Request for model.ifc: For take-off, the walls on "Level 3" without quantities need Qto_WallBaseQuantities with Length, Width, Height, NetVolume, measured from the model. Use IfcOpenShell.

First a look at what the model holds.

```python
import ifcopenshell
import ifcopenshell.util.element
import ifcopenshell.util.unit

model = ifcopenshell.open("model.ifc")
print(model.schema)
for unit_type in ("LENGTHUNIT", "AREAUNIT", "VOLUMEUNIT"):
    print(unit_type, ifcopenshell.util.unit.calculate_unit_scale(model, unit_type))
storey = next(s for s in model.by_type("IfcBuildingStorey") if s.Name == "Level 3")
walls = [e for e in ifcopenshell.util.element.get_decomposition(storey) if e.is_a("IfcWall")]
for e in sorted(walls, key=lambda e: e.id()):
    print(e.id(), e.is_a(), e.Name, list(ifcopenshell.util.element.get_psets(e, qtos_only=True)), sep=" | ")
```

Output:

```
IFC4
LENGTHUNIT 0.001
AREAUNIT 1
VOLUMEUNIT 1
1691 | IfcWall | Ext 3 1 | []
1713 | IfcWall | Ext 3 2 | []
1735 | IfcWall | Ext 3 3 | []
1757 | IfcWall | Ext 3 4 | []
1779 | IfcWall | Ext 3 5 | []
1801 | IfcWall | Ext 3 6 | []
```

```python
import ifcopenshell
import ifcopenshell.api.pset
import ifcopenshell.geom
import ifcopenshell.util.element
import ifcopenshell.util.shape
import ifcopenshell.util.unit

model = ifcopenshell.open("model.ifc")
unit_scale = ifcopenshell.util.unit.calculate_unit_scale(model)
volume_scale = ifcopenshell.util.unit.calculate_unit_scale(model, "VOLUMEUNIT")
settings = ifcopenshell.geom.settings()

storey = next(s for s in model.by_type("IfcBuildingStorey") if s.Name == "Level 3")
walls = [e for e in ifcopenshell.util.element.get_decomposition(storey) if e.is_a("IfcWall")]

for e in sorted(walls, key=lambda e: e.id()):
    if ifcopenshell.util.element.get_psets(e, qtos_only=True, should_inherit=False):
        continue
    # Geometry comes back in metres, in the element's own axes.
    shape = ifcopenshell.geom.create_shape(settings, e)
    values = {
        "Length": ifcopenshell.util.shape.get_x(shape.geometry) / unit_scale,
        "Width": ifcopenshell.util.shape.get_y(shape.geometry) / unit_scale,
        "Height": ifcopenshell.util.shape.get_z(shape.geometry) / unit_scale,
        "NetVolume": ifcopenshell.util.shape.get_volume(shape.geometry) / volume_scale,
    }
    qto = ifcopenshell.api.pset.add_qto(model, product=e, name="Qto_WallBaseQuantities")
    ifcopenshell.api.pset.edit_qto(model, qto=qto, properties=values)
    print(e.id(), {k: round(v, 3) for k, v in values.items()})

model.write("model_rev.ifc")
```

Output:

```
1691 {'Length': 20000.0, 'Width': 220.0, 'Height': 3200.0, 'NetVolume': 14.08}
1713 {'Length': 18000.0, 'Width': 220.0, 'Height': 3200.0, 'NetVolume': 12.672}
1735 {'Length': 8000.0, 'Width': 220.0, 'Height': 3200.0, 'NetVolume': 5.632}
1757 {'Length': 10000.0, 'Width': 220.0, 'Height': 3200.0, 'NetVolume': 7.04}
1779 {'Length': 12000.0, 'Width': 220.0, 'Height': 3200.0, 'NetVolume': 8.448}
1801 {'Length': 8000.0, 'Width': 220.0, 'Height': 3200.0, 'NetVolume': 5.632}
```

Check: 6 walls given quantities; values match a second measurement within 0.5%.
